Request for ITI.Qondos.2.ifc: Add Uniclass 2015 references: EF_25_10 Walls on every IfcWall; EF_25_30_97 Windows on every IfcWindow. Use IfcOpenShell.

First a look at what the model holds.

```python
import ifcopenshell

model = ifcopenshell.open("ITI.Qondos.2.ifc")
print(model.schema)
print("classifications:", [c.Name for c in model.by_type("IfcClassification")])
for ifc_class in ("IfcDoor", "IfcRoof", "IfcStair", "IfcWall", "IfcWindow"):
    print(ifc_class, len(model.by_type(ifc_class)))
```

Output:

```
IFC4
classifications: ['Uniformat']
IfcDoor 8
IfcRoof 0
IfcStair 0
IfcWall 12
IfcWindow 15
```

```python
import ifcopenshell
import ifcopenshell.api.classification

model = ifcopenshell.open("ITI.Qondos.2.ifc")

system = ifcopenshell.api.classification.add_classification(model, classification="Uniclass 2015")

codes = {
    "IfcWall": ("EF_25_10", "Walls"),
    "IfcWindow": ("EF_25_30_97", "Windows"),
}
for ifc_class, (code, name) in codes.items():
    products = model.by_type(ifc_class)
    ifcopenshell.api.classification.add_reference(
        model, products=products, classification=system, identification=code, name=name
    )
    print(code, len(products))

model.write("ITI.Qondos.2_rev.ifc")
```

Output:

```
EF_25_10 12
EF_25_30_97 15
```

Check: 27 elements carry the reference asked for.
